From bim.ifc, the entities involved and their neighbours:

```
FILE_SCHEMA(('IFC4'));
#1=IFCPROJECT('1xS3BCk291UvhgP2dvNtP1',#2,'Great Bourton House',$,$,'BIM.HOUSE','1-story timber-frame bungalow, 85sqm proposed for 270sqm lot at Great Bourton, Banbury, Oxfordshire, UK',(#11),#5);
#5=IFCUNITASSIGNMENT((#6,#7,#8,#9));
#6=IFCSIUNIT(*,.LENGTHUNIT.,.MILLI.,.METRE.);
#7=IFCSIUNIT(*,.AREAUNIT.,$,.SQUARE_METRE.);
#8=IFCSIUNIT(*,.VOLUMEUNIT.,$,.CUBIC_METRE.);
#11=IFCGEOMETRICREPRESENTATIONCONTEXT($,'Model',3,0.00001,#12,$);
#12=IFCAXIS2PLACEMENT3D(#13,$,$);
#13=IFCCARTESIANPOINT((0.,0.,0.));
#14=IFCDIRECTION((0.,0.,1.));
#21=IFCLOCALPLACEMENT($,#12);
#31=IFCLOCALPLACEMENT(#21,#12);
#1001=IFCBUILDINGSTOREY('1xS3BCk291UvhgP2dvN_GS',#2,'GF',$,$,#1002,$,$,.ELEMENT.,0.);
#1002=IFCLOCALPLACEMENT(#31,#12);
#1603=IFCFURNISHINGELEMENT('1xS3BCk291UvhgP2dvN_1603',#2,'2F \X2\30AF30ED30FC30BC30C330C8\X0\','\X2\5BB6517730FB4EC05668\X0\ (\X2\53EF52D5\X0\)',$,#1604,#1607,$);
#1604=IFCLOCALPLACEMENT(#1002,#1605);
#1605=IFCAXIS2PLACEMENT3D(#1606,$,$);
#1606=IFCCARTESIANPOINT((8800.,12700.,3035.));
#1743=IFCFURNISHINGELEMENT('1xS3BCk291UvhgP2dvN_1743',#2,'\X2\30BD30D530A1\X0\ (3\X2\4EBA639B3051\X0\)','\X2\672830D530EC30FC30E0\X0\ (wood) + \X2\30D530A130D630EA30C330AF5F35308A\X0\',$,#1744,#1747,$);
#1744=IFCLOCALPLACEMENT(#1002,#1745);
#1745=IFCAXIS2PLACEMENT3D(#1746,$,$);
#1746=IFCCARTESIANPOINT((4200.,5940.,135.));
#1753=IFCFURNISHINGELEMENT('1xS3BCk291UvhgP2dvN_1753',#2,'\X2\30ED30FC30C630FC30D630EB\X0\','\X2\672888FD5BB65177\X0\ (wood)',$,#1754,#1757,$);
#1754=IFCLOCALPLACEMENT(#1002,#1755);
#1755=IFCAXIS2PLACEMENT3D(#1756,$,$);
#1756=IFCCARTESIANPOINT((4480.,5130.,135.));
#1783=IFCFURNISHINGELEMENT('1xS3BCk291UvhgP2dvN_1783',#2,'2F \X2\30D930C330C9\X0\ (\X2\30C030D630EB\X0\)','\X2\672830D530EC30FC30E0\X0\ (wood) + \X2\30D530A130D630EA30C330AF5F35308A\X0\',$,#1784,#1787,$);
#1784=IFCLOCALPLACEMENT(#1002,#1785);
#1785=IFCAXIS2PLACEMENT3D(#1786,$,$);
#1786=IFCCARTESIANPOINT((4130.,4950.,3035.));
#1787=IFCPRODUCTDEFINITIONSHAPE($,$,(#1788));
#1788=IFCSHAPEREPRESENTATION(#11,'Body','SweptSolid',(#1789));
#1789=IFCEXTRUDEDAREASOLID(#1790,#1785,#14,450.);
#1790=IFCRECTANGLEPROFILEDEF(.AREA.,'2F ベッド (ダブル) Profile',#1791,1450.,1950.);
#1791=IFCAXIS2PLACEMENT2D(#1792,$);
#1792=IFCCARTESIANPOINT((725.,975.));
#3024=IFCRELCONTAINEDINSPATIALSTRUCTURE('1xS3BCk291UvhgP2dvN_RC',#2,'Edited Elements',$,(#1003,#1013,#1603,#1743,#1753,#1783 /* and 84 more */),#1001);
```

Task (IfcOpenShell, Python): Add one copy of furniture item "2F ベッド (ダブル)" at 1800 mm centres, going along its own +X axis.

```python
import ifcopenshell
import ifcopenshell.api.geometry
import ifcopenshell.api.root
import ifcopenshell.util.element
import ifcopenshell.util.placement
import ifcopenshell.util.unit

model = ifcopenshell.open("bim.ifc")
unit_scale = ifcopenshell.util.unit.calculate_unit_scale(model)


def reuse_history(source, copy):
    """copy_class also copies each property set's owner history, people and application; keep the originals."""
    for rel in copy.IsDefinedBy:
        if rel.is_a("IfcRelDefinesByProperties") and (history := rel.RelatingPropertyDefinition.OwnerHistory):
            rel.RelatingPropertyDefinition.OwnerHistory = source.OwnerHistory
            ifcopenshell.util.element.remove_deep2(model, history)


source = model.by_guid("1xS3BCk291UvhgP2dvN_1783")
base = ifcopenshell.util.placement.get_local_placement(source.ObjectPlacement)
step = base[:3, 0] * 1.8 / unit_scale

for i in range(1, 2):
    copy = ifcopenshell.api.root.copy_class(model, product=source)
    copy.Representation = ifcopenshell.util.element.copy_deep(
        model, source.Representation, exclude=["IfcGeometricRepresentationContext", "IfcRepresentationMap"]
    )
    reuse_history(source, copy)
    matrix = base.copy()
    matrix[:3, 3] += i * step
    print("added at", matrix[:3, 3].round(3) + 0.0)
    ifcopenshell.api.geometry.edit_object_placement(model, product=copy, matrix=matrix, is_si=False)

model.write("bim_rev.ifc")
```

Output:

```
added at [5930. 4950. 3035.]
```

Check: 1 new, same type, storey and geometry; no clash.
